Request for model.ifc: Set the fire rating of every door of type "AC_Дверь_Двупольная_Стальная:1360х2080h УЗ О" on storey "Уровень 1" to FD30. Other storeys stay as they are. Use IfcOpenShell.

First a look at what the model holds.

```python
import ifcopenshell
import ifcopenshell.util.element

model = ifcopenshell.open("model.ifc")
print(model.schema)
storey = next(s for s in model.by_type("IfcBuildingStorey") if s.Name == "Уровень 1")
doors = [e for e in ifcopenshell.util.element.get_decomposition(storey) if e.is_a("IfcDoor")]
seen = {}
for e in doors:
    element_type = ifcopenshell.util.element.get_type(e)
    key = (element_type.Name if element_type != e and element_type else None, ifcopenshell.util.element.get_pset(e, "Pset_DoorCommon", "FireRating"))
    seen[key] = seen.get(key, 0) + 1
for (name, value), count in sorted(seen.items(), key=str):
    print(count, "x", name, "|", value)
```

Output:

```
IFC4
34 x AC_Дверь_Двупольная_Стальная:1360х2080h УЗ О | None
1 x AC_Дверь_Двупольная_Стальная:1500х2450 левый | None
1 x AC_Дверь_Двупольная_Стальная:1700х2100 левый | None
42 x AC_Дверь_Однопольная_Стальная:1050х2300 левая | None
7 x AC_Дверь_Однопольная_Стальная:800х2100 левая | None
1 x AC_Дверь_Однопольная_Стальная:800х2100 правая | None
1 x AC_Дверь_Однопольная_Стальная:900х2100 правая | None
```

```python
import ifcopenshell
import ifcopenshell.api.pset
import ifcopenshell.util.element

model = ifcopenshell.open("model.ifc")

storey = next(s for s in model.by_type("IfcBuildingStorey") if s.Name == "Уровень 1")
doors = [e for e in ifcopenshell.util.element.get_decomposition(storey) if e.is_a("IfcDoor")]

count = 0
for e in doors:
    element_type = ifcopenshell.util.element.get_type(e)
    if element_type in (None, e) or element_type.Name != "AC_Дверь_Двупольная_Стальная:1360х2080h УЗ О":
        continue
    # add_pset returns the element's existing set when there is one.
    pset = ifcopenshell.api.pset.add_pset(model, product=e, name="Pset_DoorCommon")
    ifcopenshell.api.pset.edit_pset(model, pset=pset, properties={"FireRating": "FD30"})
    count += 1

print(count, "doors updated")

model.write("model-out.ifc")
```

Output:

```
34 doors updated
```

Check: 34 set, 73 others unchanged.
